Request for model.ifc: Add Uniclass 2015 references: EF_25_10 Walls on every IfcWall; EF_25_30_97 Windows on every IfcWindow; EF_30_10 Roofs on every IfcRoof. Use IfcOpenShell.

First a look at what the model holds.

```python
import ifcopenshell

model = ifcopenshell.open("model.ifc")
print(model.schema)
print("classifications:", [c.Name for c in model.by_type("IfcClassification")])
for ifc_class in ("IfcDoor", "IfcRoof", "IfcStair", "IfcWall", "IfcWindow"):
    print(ifc_class, len(model.by_type(ifc_class)))
```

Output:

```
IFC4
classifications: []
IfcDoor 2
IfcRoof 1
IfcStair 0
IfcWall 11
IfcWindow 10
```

```python
import ifcopenshell
import ifcopenshell.api.classification

model = ifcopenshell.open("model.ifc")

system = ifcopenshell.api.classification.add_classification(model, classification="Uniclass 2015")

codes = {
    "IfcWall": ("EF_25_10", "Walls"),
    "IfcWindow": ("EF_25_30_97", "Windows"),
    "IfcRoof": ("EF_30_10", "Roofs"),
}
for ifc_class, (code, name) in codes.items():
    products = model.by_type(ifc_class)
    ifcopenshell.api.classification.add_reference(
        model, products=products, classification=system, identification=code, name=name
    )
    print(code, len(products))

model.write("model_v2.ifc")
```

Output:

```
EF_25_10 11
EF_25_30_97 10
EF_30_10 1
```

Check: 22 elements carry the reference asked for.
